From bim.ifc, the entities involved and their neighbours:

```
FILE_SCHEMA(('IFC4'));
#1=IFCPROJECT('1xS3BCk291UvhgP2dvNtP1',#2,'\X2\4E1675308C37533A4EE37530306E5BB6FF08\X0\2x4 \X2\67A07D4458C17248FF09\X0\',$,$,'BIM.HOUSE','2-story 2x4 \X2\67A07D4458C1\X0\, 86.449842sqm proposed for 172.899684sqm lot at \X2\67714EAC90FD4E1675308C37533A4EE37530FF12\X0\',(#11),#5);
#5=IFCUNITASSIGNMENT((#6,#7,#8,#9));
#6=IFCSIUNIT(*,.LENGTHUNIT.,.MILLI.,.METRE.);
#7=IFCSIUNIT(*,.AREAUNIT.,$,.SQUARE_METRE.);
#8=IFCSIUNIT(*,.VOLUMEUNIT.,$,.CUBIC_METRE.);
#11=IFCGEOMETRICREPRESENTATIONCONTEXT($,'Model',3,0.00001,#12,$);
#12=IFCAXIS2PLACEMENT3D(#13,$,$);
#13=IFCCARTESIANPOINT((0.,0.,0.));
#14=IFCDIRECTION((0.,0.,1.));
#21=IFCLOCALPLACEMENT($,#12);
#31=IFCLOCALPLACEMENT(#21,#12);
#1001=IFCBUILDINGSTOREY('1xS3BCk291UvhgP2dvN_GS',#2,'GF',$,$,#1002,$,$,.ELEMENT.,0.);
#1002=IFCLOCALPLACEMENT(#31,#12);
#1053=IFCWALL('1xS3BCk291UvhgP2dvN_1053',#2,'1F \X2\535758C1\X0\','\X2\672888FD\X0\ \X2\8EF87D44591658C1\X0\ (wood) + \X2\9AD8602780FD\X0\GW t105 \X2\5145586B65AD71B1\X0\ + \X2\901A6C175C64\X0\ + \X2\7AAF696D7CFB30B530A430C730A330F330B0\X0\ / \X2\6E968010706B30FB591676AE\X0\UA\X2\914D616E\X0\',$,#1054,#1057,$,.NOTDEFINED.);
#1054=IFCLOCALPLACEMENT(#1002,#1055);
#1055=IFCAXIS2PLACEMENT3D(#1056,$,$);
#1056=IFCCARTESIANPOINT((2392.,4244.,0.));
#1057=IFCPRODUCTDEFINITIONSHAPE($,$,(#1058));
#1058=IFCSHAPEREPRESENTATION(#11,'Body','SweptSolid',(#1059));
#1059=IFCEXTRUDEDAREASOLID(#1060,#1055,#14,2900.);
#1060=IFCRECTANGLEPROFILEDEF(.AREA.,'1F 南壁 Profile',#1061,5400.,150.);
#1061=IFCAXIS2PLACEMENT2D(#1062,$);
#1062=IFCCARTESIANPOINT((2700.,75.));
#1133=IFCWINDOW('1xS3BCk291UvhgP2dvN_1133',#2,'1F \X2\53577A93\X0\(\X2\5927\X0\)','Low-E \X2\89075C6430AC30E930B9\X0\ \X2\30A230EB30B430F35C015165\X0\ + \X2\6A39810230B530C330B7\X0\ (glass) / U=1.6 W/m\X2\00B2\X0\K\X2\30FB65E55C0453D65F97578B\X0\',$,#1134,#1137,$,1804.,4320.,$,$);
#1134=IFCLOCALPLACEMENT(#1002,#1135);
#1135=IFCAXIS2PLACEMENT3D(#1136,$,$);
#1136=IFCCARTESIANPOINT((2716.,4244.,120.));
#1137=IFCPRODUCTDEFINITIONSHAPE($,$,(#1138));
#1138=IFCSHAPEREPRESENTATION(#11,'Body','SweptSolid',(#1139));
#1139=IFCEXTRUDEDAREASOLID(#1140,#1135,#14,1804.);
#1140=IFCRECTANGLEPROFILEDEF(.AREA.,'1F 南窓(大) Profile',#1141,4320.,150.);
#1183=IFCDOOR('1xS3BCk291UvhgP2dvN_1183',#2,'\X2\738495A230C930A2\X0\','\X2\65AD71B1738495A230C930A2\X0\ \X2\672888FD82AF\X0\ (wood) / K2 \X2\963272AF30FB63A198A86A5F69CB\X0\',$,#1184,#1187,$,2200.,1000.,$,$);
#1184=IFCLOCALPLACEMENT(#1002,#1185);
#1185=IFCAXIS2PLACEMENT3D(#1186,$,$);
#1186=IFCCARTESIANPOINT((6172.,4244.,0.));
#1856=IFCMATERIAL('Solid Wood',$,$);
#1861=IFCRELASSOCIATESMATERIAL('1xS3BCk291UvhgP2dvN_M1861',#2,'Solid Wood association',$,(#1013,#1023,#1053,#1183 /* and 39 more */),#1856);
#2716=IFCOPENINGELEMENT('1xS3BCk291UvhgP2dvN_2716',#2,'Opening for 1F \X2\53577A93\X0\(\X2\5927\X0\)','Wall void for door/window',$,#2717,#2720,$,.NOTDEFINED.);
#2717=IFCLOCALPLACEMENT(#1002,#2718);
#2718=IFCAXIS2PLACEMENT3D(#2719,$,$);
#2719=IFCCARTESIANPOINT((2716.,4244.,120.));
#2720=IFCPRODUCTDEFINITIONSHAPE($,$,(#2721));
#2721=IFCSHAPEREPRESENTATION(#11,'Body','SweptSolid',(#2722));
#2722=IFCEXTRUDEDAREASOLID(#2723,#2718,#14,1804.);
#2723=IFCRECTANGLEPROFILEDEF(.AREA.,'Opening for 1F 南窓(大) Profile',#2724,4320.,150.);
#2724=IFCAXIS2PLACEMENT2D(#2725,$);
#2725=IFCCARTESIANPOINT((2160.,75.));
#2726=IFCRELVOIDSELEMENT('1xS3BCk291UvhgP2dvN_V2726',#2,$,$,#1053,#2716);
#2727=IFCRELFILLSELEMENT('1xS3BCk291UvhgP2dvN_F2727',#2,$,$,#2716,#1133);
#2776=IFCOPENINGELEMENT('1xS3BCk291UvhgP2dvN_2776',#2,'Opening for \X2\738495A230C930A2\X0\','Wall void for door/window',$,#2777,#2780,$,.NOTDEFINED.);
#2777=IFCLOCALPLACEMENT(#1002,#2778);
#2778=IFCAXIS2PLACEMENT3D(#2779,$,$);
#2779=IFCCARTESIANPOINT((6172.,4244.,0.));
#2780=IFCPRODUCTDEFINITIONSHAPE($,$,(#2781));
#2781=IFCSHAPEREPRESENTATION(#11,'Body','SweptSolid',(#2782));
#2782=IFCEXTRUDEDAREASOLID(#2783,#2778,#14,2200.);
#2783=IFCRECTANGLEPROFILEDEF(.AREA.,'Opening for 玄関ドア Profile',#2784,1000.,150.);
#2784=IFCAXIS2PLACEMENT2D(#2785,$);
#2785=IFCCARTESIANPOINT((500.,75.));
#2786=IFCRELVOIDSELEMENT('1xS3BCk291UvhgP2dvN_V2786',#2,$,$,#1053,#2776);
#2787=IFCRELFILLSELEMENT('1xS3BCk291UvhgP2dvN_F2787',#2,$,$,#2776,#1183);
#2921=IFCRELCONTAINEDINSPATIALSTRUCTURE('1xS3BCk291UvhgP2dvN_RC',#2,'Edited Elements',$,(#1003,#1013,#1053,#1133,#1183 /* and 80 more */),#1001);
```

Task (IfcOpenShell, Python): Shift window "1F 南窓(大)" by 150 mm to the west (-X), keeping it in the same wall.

```python
import ifcopenshell
import ifcopenshell.api.geometry
import ifcopenshell.util.placement
import ifcopenshell.util.unit

model = ifcopenshell.open("bim.ifc")
unit_scale = ifcopenshell.util.unit.calculate_unit_scale(model)

window = model.by_guid("1xS3BCk291UvhgP2dvN_1133")
opening = window.FillsVoids[0].RelatingOpeningElement
wall = opening.VoidsElements[0].RelatingBuildingElement

wall_matrix = ifcopenshell.util.placement.get_local_placement(wall.ObjectPlacement)
shift = wall_matrix[:3, 0] * -0.15 / unit_scale
before = ifcopenshell.util.placement.get_local_placement(window.ObjectPlacement)[:3, 3].copy()

# The window is not placed relative to its opening, so move both.
for product in (opening, window):
    matrix = ifcopenshell.util.placement.get_local_placement(product.ObjectPlacement)
    matrix[:3, 3] += shift
    ifcopenshell.api.geometry.edit_object_placement(model, product=product, matrix=matrix, is_si=False)

after = ifcopenshell.util.placement.get_local_placement(window.ObjectPlacement)[:3, 3]
print("window moved by", (after - before).round(3) + 0.0)

model.write("bim_rev.ifc")
```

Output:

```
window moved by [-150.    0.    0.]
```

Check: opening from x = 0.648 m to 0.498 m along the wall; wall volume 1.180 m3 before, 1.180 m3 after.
